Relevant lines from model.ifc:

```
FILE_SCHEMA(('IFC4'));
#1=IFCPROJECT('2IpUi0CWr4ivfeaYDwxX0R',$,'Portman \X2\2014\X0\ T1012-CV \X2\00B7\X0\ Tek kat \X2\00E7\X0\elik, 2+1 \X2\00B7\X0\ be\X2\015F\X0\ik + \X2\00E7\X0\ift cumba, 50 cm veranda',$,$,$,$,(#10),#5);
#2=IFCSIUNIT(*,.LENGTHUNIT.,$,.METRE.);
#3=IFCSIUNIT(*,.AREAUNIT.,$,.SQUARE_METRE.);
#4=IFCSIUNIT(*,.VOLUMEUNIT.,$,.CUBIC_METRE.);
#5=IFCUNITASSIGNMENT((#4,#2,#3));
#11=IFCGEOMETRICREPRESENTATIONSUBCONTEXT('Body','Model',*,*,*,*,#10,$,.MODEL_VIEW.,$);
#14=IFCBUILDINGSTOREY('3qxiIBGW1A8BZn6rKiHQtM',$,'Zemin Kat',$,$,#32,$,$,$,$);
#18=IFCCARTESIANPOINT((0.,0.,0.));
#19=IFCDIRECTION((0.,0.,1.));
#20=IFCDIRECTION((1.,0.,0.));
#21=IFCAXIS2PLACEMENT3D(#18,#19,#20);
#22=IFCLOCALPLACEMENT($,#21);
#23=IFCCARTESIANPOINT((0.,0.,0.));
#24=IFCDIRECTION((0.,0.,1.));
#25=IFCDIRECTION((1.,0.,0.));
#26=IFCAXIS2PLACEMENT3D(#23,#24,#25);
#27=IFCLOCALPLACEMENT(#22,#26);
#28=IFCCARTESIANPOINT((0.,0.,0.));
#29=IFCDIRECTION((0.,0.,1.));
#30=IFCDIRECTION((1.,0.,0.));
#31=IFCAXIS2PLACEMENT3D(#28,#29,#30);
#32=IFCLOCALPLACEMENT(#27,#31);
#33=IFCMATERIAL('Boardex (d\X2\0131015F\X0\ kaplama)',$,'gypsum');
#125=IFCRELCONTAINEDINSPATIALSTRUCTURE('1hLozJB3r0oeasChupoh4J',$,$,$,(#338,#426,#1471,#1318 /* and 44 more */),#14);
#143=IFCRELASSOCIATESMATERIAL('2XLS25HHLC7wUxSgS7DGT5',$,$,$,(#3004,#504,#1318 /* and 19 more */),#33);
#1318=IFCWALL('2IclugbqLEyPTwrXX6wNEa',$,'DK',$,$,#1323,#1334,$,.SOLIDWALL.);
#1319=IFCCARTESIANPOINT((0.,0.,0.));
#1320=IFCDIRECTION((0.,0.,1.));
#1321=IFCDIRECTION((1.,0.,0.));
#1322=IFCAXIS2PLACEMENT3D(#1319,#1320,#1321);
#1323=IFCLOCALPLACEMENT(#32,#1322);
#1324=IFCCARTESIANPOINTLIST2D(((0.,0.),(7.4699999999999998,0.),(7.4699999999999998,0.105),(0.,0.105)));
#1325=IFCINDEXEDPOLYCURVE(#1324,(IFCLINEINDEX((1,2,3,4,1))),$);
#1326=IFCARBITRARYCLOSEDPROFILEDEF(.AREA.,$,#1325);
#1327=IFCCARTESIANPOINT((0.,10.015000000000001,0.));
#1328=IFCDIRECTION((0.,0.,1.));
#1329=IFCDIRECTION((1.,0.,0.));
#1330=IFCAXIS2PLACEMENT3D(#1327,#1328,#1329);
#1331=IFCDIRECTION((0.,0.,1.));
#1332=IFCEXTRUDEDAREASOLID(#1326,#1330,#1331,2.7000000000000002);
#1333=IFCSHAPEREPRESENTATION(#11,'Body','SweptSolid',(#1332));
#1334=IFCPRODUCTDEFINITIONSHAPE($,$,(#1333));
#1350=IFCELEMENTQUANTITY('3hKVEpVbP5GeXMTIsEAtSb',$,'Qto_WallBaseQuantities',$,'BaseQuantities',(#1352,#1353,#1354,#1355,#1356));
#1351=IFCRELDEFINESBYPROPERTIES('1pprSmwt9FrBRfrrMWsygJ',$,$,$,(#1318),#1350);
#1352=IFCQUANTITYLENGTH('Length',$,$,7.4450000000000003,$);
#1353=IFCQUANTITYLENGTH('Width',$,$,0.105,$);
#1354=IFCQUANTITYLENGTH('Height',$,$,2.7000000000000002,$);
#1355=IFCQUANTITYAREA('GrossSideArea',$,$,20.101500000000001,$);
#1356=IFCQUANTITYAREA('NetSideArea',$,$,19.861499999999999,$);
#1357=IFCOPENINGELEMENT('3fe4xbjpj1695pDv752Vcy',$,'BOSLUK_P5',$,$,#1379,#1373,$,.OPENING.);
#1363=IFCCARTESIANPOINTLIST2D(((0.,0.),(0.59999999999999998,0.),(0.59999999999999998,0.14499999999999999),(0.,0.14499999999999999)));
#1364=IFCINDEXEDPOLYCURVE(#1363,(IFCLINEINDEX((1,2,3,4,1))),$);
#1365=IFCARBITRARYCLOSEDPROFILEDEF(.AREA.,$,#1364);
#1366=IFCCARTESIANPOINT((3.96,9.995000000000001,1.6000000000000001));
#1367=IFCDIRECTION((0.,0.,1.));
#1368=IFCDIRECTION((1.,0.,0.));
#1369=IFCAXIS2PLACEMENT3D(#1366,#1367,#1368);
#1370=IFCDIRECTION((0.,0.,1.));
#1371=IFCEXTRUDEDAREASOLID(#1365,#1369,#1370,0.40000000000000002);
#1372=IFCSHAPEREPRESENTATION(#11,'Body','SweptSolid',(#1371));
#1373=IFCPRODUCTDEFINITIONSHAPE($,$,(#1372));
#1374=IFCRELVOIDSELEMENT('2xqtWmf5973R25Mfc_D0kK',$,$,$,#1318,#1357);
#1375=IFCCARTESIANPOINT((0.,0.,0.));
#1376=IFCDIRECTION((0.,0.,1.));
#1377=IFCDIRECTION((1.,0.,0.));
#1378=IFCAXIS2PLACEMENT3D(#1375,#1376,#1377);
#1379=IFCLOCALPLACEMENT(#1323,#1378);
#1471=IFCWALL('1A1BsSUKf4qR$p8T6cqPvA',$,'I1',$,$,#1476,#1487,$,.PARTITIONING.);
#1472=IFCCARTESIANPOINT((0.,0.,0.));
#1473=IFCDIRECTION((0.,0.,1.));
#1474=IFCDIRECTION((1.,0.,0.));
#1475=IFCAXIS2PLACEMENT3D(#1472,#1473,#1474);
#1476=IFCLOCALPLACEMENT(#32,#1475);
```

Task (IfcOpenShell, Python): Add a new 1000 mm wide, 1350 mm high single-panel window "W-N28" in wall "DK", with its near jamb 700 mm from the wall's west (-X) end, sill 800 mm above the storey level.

```python
import numpy as np
import ifcopenshell
import ifcopenshell.api.feature
import ifcopenshell.api.geometry
import ifcopenshell.api.pset
import ifcopenshell.api.root
import ifcopenshell.api.spatial
import ifcopenshell.geom
import ifcopenshell.util.element
import ifcopenshell.util.placement
import ifcopenshell.util.representation
import ifcopenshell.util.shape
import ifcopenshell.util.unit

model = ifcopenshell.open("model.ifc")
unit_scale = ifcopenshell.util.unit.calculate_unit_scale(model)
area_scale = ifcopenshell.util.unit.calculate_unit_scale(model, "AREAUNIT")
settings = ifcopenshell.geom.settings()


def volume(element):
    """Net volume in cubic metres, openings subtracted."""
    shape = ifcopenshell.geom.create_shape(settings, element)
    return ifcopenshell.util.shape.get_volume(shape.geometry)


wall = model.by_id(1318)
storey = ifcopenshell.util.element.get_container(wall, ifc_class="IfcBuildingStorey")
context = ifcopenshell.util.representation.get_context(model, "Model", "Body", "MODEL_VIEW")
before = volume(wall)

width, height, from_end, sill = 1, 1.35, 0.7, 0.8  # metres

# The wall runs along its own X axis, and the end named is its -X end.
wall_shape = ifcopenshell.geom.create_shape(settings, wall)
x, y, z = ifcopenshell.util.shape.get_vertices(wall_shape.geometry).T
start = x.min() + from_end
face, thickness = float(y.min()), float(y.max() - y.min())
wall_matrix = ifcopenshell.util.placement.get_local_placement(wall.ObjectPlacement)
level = ifcopenshell.util.placement.get_local_placement(storey.ObjectPlacement)[2, 3]


def in_wall(x, y):
    """Placement at x, y metres in the wall's axes, at sill height."""
    matrix = wall_matrix.copy()
    matrix[:, 3] = wall_matrix @ np.array([x / unit_scale, y / unit_scale, 0.0, 1.0])
    matrix[2, 3] = level + sill / unit_scale
    return matrix


# Opening: a box that overshoots both wall faces by 50 mm.
opening = ifcopenshell.api.root.create_entity(model, ifc_class="IfcOpeningElement", predefined_type="OPENING")
box = ifcopenshell.api.geometry.add_wall_representation(
    model, context=context, length=width, height=height, thickness=thickness + 0.1
)
ifcopenshell.api.geometry.assign_representation(model, product=opening, representation=box)
ifcopenshell.api.geometry.edit_object_placement(model, product=opening, matrix=in_wall(start, face - 0.05), is_si=False)
ifcopenshell.api.feature.add_feature(model, feature=opening, element=wall)

window = ifcopenshell.api.root.create_entity(model, ifc_class="IfcWindow", name="W-N28", predefined_type="WINDOW")
window.OverallWidth, window.OverallHeight = width / unit_scale, height / unit_scale
window.PartitioningType = "SINGLE_PANEL"
body = ifcopenshell.api.geometry.add_window_representation(
    model,
    context=context,
    overall_width=window.OverallWidth,
    overall_height=window.OverallHeight,
    partition_type="SINGLE_PANEL",
)
ifcopenshell.api.geometry.assign_representation(model, product=window, representation=body)
ifcopenshell.api.spatial.assign_container(model, products=[window], relating_structure=storey)
ifcopenshell.api.feature.add_filling(model, opening=opening, element=window)

# Centre the window in the wall's thickness.
ifcopenshell.api.geometry.edit_object_placement(model, product=window, matrix=in_wall(start, face), is_si=False)
window_shape = ifcopenshell.geom.create_shape(settings, window)
depth = ifcopenshell.util.shape.get_vertices(window_shape.geometry)[:, 1]
offset = face + thickness / 2 - (depth.min() + depth.max()) / 2
ifcopenshell.api.geometry.edit_object_placement(model, product=window, matrix=in_wall(start, offset), is_si=False)

after = volume(wall)

# Update the wall's stored quantities.
qto = model.by_id(ifcopenshell.util.element.get_pset(wall, "Qto_WallBaseQuantities", should_inherit=False)["id"])
ifcopenshell.api.pset.edit_qto(model, qto=qto, properties={"NetSideArea": after / thickness / area_scale})

print(f"wall volume {before:.3f} -> {after:.3f} m3")

model.write("model_rev.ifc")
```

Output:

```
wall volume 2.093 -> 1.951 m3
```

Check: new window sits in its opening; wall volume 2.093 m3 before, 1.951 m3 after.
